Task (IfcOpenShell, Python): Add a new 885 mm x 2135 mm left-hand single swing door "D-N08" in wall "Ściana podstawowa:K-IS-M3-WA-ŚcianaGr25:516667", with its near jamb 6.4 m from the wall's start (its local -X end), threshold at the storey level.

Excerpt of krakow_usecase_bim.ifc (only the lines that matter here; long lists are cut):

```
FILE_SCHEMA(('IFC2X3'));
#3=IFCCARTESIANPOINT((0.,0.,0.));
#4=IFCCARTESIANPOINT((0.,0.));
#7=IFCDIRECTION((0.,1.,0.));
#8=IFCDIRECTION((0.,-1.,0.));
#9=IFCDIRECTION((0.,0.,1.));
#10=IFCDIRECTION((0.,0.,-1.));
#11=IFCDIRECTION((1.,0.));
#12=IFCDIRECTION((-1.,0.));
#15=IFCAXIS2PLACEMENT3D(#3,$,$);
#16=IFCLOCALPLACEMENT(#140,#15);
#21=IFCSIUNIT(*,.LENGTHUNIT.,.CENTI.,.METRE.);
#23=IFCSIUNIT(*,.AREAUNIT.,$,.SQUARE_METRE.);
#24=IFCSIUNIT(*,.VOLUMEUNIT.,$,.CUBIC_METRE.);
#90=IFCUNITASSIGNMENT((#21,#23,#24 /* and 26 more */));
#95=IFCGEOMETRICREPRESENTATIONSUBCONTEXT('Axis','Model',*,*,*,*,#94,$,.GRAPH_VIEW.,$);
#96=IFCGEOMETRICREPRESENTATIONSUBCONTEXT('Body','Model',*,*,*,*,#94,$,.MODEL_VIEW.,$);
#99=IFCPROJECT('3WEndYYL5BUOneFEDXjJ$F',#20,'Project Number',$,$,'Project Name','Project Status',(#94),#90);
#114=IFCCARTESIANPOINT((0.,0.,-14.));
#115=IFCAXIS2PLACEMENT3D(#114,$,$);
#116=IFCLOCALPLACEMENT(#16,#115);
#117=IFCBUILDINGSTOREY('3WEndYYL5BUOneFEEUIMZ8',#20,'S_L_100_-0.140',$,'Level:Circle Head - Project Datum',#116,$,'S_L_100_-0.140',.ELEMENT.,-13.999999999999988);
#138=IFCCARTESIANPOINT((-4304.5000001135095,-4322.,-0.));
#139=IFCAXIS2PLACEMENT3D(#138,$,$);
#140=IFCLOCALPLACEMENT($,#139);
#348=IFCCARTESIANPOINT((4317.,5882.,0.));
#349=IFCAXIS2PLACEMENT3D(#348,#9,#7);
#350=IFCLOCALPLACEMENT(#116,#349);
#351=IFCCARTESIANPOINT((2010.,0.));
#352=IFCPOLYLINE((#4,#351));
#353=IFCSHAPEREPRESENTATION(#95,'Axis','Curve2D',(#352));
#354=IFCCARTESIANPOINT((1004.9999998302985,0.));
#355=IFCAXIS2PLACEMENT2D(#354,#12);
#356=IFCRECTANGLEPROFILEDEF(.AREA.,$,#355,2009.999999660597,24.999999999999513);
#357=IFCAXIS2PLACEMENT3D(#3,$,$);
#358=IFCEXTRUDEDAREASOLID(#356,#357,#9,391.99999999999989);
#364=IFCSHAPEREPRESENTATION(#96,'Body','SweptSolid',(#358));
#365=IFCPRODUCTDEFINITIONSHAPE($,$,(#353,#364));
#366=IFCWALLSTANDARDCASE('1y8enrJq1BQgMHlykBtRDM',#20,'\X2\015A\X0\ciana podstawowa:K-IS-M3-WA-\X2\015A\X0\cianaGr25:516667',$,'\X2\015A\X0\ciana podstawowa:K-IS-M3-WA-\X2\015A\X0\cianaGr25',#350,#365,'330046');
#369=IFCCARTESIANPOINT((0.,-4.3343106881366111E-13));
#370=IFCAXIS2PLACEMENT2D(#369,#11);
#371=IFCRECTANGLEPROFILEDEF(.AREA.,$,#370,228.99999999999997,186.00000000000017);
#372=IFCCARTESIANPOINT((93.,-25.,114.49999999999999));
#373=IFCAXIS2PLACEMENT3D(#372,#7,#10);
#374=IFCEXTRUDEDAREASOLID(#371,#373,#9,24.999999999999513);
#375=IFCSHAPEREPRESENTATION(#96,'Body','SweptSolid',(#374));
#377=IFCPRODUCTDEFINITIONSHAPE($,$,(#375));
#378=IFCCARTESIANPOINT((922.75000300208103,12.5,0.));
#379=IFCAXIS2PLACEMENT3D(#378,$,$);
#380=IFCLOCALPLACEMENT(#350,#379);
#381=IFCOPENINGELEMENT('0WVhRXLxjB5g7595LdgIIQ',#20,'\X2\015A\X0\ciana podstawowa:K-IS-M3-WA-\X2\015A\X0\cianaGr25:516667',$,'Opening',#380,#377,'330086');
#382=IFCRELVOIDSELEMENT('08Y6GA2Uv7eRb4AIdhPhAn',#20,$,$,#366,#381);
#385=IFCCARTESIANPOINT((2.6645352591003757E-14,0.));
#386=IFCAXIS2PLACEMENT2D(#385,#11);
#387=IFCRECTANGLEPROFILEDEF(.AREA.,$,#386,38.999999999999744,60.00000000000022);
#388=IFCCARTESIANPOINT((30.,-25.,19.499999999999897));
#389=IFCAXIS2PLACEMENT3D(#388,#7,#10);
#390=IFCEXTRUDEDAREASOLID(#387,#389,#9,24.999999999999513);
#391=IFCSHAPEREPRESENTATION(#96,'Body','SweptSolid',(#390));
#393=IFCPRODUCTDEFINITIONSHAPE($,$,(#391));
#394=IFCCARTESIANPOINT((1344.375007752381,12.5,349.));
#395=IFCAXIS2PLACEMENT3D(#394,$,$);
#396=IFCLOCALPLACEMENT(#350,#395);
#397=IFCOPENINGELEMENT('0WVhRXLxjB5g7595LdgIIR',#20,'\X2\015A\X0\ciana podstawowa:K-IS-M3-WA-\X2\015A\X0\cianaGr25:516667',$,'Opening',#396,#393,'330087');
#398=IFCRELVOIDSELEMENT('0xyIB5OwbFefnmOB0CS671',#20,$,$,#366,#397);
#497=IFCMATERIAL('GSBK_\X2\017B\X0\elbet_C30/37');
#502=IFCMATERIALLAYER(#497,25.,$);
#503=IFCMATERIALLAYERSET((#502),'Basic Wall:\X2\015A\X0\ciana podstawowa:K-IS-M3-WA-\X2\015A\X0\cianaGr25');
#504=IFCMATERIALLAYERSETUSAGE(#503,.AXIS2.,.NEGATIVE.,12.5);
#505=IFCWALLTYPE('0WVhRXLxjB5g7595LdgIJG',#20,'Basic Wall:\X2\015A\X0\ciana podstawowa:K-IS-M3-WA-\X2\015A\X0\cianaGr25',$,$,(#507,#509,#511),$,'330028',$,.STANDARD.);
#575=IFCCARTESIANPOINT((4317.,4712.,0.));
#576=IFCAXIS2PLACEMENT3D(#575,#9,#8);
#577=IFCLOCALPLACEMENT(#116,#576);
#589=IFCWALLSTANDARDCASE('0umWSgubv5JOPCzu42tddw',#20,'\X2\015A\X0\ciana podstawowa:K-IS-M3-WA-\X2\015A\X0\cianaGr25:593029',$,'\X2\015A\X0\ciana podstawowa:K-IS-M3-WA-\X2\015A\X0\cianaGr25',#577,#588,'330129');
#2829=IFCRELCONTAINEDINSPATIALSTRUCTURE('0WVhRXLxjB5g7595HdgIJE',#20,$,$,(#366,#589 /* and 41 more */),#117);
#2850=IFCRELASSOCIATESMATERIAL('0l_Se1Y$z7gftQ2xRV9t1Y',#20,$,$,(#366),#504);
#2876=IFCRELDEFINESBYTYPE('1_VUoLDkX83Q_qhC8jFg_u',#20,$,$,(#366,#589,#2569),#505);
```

```python
import numpy as np
import ifcopenshell
import ifcopenshell.api.feature
import ifcopenshell.api.geometry
import ifcopenshell.api.root
import ifcopenshell.api.spatial
import ifcopenshell.api.type
import ifcopenshell.geom
import ifcopenshell.util.element
import ifcopenshell.util.placement
import ifcopenshell.util.representation
import ifcopenshell.util.shape
import ifcopenshell.util.unit

model = ifcopenshell.open("krakow_usecase_bim.ifc")
unit_scale = ifcopenshell.util.unit.calculate_unit_scale(model)
settings = ifcopenshell.geom.settings()


def volume(element):
    """Net volume in cubic metres, openings subtracted."""
    shape = ifcopenshell.geom.create_shape(settings, element)
    return ifcopenshell.util.shape.get_volume(shape.geometry)


wall = model.by_guid("1y8enrJq1BQgMHlykBtRDM")
storey = ifcopenshell.util.element.get_container(wall, ifc_class="IfcBuildingStorey")
context = ifcopenshell.util.representation.get_context(model, "Model", "Body", "MODEL_VIEW")
before = volume(wall)

width, height, from_end, sill = 0.885, 2.135, 6.4, 0.0  # metres

# The wall runs along its own X axis, and the end named is its -X end.
wall_shape = ifcopenshell.geom.create_shape(settings, wall)
x, y, z = ifcopenshell.util.shape.get_vertices(wall_shape.geometry).T
start = x.min() + from_end
face, thickness = float(y.min()), float(y.max() - y.min())
wall_matrix = ifcopenshell.util.placement.get_local_placement(wall.ObjectPlacement)
level = ifcopenshell.util.placement.get_local_placement(storey.ObjectPlacement)[2, 3]


def in_wall(x, y):
    """Placement at x, y metres in the wall's axes, at sill height."""
    matrix = wall_matrix.copy()
    matrix[:, 3] = wall_matrix @ np.array([x / unit_scale, y / unit_scale, 0.0, 1.0])
    matrix[2, 3] = level + sill / unit_scale
    return matrix


# Opening: a box that overshoots both wall faces by 50 mm.
opening = ifcopenshell.api.root.create_entity(model, ifc_class="IfcOpeningElement")
box = ifcopenshell.api.geometry.add_wall_representation(
    model, context=context, length=width, height=height, thickness=thickness + 0.1
)
ifcopenshell.api.geometry.assign_representation(model, product=opening, representation=box)
ifcopenshell.api.geometry.edit_object_placement(model, product=opening, matrix=in_wall(start, face - 0.05), is_si=False)
ifcopenshell.api.feature.add_feature(model, feature=opening, element=wall)

door = ifcopenshell.api.root.create_entity(model, ifc_class="IfcDoor", name="D-N08")
door.OverallWidth, door.OverallHeight = width / unit_scale, height / unit_scale
body = ifcopenshell.api.geometry.add_door_representation(
    model,
    context=context,
    overall_width=door.OverallWidth,
    overall_height=door.OverallHeight,
    operation_type="SINGLE_SWING_LEFT",
    lining_properties={"LiningDepth": thickness / unit_scale, "ThresholdDepth": thickness / unit_scale},
)
ifcopenshell.api.geometry.assign_representation(model, product=door, representation=body)
ifcopenshell.api.spatial.assign_container(model, products=[door], relating_structure=storey)
fills = ifcopenshell.api.feature.add_filling(model, opening=opening, element=door)
fills.OwnerHistory = door.OwnerHistory  # required in IFC2X3

# IFC2X3 keeps the operation on the door style.
style = ifcopenshell.api.root.create_entity(model, ifc_class="IfcDoorStyle", name="D-N08")
style.OperationType, style.ConstructionType = "SINGLE_SWING_LEFT", "NOTDEFINED"
style.ParameterTakesPrecedence = style.Sizeable = False
ifcopenshell.api.type.assign_type(model, related_objects=[door], relating_type=style)

# The lining spans the wall, so the door starts at the wall face.
ifcopenshell.api.geometry.edit_object_placement(model, product=door, matrix=in_wall(start, face), is_si=False)

after = volume(wall)

print(f"wall volume {before:.3f} -> {after:.3f} m3")

model.write("krakow_usecase_bim-out.ifc")
```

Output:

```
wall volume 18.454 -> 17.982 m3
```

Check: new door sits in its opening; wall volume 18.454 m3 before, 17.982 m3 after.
